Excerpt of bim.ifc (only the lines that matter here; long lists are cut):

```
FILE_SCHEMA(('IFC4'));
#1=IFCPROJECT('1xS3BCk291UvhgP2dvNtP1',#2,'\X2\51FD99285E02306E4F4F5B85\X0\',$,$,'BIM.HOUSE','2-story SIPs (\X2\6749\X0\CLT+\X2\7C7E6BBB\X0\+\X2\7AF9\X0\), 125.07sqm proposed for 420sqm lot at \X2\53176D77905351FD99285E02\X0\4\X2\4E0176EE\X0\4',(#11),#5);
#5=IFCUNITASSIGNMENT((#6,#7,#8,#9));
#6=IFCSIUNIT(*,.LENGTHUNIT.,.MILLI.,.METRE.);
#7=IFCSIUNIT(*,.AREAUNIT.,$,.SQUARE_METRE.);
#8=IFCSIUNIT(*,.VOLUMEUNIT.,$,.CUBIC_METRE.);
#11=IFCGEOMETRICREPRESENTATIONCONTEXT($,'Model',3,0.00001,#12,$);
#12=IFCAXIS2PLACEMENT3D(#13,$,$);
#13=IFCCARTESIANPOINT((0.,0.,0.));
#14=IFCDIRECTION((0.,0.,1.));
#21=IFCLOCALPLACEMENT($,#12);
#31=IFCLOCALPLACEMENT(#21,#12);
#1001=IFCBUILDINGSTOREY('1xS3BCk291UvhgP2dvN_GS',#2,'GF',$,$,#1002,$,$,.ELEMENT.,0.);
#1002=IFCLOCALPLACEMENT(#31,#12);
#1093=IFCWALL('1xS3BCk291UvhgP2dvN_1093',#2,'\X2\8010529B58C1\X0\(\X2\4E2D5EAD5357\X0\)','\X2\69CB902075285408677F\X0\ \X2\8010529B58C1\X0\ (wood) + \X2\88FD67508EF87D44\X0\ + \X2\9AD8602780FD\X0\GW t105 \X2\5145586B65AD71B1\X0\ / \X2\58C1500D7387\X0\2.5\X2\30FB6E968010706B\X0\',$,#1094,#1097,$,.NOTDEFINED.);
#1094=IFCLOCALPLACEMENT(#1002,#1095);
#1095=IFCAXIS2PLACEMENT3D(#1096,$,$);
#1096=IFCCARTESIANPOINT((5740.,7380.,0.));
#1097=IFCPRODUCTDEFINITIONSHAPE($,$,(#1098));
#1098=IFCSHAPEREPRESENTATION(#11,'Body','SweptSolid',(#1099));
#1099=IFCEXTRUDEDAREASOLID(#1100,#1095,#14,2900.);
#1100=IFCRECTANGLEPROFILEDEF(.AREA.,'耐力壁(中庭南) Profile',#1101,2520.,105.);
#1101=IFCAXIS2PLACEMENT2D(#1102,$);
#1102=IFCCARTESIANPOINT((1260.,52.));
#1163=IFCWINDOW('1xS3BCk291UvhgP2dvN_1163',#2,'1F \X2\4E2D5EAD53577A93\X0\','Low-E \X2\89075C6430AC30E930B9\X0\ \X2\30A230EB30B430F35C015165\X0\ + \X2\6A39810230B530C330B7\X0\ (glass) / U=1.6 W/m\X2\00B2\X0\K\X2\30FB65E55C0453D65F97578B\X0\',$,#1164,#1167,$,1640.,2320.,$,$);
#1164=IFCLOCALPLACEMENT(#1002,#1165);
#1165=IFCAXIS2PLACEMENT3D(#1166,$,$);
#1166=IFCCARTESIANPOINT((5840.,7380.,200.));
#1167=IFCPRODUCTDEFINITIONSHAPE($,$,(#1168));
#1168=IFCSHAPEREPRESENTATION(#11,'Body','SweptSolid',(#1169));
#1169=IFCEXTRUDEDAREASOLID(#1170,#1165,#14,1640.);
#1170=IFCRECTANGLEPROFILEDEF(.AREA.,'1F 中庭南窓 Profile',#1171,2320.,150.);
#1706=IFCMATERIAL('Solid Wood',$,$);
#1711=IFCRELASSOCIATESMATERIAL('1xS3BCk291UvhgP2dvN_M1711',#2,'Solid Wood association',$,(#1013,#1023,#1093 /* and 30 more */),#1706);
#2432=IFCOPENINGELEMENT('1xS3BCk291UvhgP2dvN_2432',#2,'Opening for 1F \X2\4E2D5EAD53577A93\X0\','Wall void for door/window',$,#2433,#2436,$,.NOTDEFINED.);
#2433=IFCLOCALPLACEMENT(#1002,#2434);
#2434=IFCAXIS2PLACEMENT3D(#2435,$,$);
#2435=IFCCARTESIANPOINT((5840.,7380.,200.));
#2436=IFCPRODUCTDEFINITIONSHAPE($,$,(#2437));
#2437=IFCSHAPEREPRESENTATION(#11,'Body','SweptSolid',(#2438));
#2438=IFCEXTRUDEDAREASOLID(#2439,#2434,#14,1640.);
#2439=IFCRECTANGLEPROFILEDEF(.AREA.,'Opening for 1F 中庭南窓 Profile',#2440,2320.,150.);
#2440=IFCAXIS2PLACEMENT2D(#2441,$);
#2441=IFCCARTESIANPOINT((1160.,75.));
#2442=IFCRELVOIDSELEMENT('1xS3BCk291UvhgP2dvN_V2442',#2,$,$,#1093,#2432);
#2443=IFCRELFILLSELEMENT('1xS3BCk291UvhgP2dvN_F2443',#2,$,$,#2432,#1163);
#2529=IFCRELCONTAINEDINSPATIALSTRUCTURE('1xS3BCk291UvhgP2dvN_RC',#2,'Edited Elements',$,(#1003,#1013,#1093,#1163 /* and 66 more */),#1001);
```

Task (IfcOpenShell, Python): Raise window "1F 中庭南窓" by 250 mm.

```python
import numpy as np
import ifcopenshell
import ifcopenshell.api.geometry
import ifcopenshell.util.placement
import ifcopenshell.util.unit

model = ifcopenshell.open("bim.ifc")
unit_scale = ifcopenshell.util.unit.calculate_unit_scale(model)

window = model.by_id(1163)
opening = window.FillsVoids[0].RelatingOpeningElement
dz = 0.25 / unit_scale

shift = np.array([0.0, 0.0, dz])
# The window is not placed relative to its opening, so move both.
for product in (opening, window):
    matrix = ifcopenshell.util.placement.get_local_placement(product.ObjectPlacement)
    matrix[:3, 3] += shift
    ifcopenshell.api.geometry.edit_object_placement(model, product=product, matrix=matrix, is_si=False)

print(f"moved by {dz * unit_scale:+.3f} m")

model.write("bim_edited.ifc")
```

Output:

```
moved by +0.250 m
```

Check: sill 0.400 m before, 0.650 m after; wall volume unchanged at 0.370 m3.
